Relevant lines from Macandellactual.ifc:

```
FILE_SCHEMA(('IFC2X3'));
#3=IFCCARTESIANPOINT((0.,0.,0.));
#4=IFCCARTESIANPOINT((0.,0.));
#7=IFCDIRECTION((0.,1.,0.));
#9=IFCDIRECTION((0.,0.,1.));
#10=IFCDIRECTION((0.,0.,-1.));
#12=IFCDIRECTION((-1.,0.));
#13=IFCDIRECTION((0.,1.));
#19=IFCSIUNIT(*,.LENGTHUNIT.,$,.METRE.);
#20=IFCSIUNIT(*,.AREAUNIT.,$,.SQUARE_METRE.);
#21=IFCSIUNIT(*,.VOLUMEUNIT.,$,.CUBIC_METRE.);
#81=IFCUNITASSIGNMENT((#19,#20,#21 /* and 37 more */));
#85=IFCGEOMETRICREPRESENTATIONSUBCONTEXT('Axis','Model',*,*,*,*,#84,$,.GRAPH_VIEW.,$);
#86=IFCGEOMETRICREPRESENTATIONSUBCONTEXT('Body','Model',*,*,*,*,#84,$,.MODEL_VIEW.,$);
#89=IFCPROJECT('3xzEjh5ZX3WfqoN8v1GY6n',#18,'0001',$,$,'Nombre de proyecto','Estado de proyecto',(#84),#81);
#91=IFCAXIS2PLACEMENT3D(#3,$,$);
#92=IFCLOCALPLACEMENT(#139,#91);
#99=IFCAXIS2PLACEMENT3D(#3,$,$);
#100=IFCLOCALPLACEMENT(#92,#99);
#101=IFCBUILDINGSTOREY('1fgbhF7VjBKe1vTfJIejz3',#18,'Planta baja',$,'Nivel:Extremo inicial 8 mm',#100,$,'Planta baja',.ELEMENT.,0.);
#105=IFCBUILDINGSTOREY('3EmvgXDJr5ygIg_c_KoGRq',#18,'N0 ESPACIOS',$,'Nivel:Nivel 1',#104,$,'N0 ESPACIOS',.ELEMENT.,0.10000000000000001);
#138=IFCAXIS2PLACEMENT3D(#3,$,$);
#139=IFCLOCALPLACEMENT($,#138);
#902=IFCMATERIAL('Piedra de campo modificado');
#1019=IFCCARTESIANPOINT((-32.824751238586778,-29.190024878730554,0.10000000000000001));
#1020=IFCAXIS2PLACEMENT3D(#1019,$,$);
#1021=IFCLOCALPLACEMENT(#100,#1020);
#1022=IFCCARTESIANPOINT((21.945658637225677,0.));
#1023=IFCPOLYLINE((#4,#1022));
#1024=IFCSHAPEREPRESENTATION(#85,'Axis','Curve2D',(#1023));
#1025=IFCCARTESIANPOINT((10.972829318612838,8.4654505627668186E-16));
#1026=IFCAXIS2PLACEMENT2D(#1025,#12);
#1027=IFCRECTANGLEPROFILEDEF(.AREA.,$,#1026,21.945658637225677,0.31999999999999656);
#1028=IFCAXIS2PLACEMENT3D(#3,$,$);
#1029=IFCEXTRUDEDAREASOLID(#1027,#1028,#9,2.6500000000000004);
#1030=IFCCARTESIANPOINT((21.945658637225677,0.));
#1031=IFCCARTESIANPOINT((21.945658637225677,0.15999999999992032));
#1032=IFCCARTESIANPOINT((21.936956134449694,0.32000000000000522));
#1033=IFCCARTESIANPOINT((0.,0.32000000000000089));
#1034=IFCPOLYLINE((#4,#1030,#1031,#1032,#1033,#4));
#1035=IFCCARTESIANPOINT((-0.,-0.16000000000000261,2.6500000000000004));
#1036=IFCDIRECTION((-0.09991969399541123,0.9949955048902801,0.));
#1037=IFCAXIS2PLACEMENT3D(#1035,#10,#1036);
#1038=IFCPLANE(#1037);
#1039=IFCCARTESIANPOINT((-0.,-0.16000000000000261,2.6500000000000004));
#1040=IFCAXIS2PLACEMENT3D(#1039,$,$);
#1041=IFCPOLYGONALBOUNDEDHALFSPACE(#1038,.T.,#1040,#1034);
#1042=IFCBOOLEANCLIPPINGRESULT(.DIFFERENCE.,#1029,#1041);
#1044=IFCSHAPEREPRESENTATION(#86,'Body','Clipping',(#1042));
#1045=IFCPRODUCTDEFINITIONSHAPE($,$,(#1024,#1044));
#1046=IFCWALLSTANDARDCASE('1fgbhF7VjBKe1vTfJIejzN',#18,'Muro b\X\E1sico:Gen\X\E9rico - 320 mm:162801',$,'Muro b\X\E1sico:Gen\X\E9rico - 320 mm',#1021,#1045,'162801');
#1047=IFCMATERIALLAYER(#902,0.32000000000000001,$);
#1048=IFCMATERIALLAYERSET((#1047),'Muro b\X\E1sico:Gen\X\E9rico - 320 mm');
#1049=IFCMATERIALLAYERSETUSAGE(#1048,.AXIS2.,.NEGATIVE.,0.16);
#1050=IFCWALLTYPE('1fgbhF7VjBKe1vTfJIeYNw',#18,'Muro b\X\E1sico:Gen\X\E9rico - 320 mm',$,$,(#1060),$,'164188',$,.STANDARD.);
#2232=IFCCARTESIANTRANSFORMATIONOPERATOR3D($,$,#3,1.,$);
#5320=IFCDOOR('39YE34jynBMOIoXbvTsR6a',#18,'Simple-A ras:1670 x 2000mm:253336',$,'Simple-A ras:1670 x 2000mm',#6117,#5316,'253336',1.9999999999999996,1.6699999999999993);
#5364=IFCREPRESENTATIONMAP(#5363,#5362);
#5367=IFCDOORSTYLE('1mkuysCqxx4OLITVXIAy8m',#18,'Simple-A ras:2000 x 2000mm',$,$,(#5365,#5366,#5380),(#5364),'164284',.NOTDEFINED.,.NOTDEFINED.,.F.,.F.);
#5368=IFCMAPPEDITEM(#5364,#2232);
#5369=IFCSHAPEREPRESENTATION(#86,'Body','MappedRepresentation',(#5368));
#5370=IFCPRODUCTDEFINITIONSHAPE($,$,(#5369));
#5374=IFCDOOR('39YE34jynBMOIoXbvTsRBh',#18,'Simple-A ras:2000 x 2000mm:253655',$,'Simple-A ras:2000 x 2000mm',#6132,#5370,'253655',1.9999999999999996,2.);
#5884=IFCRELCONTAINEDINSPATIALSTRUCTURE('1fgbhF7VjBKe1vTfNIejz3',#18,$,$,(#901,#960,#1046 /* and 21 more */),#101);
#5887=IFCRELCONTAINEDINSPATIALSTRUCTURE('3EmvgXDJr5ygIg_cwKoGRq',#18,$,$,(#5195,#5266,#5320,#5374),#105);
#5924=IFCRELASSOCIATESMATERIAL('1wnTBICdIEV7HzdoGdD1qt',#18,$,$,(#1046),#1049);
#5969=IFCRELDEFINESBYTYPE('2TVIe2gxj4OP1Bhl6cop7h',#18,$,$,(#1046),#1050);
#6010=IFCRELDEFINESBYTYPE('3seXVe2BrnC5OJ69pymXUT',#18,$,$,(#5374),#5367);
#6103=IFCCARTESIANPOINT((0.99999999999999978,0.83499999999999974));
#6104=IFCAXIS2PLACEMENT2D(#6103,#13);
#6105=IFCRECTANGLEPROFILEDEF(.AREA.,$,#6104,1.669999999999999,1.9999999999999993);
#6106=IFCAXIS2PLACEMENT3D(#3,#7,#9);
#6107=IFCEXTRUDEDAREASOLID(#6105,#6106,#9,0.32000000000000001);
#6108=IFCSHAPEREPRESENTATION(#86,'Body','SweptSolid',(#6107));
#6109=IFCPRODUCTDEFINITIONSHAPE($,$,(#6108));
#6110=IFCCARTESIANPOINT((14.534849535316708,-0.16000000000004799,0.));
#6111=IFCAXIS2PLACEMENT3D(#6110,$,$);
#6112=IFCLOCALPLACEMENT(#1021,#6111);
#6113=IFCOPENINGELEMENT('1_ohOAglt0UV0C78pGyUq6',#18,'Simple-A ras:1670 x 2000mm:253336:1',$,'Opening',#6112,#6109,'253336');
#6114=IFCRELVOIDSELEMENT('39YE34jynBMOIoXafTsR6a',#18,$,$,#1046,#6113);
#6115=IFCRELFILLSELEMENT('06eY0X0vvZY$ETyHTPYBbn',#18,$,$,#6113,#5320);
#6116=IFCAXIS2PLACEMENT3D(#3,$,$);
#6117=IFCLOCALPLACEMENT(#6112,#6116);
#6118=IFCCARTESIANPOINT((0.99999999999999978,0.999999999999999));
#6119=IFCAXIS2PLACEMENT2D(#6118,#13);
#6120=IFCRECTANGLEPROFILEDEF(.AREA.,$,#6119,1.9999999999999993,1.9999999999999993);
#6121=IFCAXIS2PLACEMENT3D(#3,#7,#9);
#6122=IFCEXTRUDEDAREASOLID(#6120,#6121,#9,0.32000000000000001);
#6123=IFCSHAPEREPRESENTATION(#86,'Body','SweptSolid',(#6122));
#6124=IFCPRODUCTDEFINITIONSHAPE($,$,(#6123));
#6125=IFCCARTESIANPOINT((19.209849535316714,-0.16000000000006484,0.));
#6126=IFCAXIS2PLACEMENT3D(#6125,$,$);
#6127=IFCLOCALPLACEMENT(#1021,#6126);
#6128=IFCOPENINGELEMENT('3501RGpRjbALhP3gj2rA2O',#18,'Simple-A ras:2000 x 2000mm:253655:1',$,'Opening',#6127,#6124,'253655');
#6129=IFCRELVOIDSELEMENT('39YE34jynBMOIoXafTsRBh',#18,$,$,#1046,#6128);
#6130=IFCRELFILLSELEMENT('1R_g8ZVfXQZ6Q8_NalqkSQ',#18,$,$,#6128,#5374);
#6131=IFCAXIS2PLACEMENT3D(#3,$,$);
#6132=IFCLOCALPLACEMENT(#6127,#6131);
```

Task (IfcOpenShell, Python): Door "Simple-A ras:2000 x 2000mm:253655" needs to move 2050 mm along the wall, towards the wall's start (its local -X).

```python
import ifcopenshell
import ifcopenshell.api.geometry
import ifcopenshell.util.placement

model = ifcopenshell.open("Macandellactual.ifc")

door = model.by_guid("39YE34jynBMOIoXbvTsRBh")
opening = door.FillsVoids[0].RelatingOpeningElement
wall = opening.VoidsElements[0].RelatingBuildingElement

wall_matrix = ifcopenshell.util.placement.get_local_placement(wall.ObjectPlacement)
shift = wall_matrix[:3, 0] * -2.05
before = ifcopenshell.util.placement.get_local_placement(door.ObjectPlacement)[:3, 3].copy()

# The door is placed relative to its opening, so it follows when the opening moves.
matrix = ifcopenshell.util.placement.get_local_placement(opening.ObjectPlacement)
matrix[:3, 3] += shift
ifcopenshell.api.geometry.edit_object_placement(
    model, product=opening, matrix=matrix, is_si=False, should_transform_children=True
)

after = ifcopenshell.util.placement.get_local_placement(door.ObjectPlacement)[:3, 3]
print("door moved by", (after - before).round(3) + 0.0)

model.write("Macandellactual_updated.ifc")
```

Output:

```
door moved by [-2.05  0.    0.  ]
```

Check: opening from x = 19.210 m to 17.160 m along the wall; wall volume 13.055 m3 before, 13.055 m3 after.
